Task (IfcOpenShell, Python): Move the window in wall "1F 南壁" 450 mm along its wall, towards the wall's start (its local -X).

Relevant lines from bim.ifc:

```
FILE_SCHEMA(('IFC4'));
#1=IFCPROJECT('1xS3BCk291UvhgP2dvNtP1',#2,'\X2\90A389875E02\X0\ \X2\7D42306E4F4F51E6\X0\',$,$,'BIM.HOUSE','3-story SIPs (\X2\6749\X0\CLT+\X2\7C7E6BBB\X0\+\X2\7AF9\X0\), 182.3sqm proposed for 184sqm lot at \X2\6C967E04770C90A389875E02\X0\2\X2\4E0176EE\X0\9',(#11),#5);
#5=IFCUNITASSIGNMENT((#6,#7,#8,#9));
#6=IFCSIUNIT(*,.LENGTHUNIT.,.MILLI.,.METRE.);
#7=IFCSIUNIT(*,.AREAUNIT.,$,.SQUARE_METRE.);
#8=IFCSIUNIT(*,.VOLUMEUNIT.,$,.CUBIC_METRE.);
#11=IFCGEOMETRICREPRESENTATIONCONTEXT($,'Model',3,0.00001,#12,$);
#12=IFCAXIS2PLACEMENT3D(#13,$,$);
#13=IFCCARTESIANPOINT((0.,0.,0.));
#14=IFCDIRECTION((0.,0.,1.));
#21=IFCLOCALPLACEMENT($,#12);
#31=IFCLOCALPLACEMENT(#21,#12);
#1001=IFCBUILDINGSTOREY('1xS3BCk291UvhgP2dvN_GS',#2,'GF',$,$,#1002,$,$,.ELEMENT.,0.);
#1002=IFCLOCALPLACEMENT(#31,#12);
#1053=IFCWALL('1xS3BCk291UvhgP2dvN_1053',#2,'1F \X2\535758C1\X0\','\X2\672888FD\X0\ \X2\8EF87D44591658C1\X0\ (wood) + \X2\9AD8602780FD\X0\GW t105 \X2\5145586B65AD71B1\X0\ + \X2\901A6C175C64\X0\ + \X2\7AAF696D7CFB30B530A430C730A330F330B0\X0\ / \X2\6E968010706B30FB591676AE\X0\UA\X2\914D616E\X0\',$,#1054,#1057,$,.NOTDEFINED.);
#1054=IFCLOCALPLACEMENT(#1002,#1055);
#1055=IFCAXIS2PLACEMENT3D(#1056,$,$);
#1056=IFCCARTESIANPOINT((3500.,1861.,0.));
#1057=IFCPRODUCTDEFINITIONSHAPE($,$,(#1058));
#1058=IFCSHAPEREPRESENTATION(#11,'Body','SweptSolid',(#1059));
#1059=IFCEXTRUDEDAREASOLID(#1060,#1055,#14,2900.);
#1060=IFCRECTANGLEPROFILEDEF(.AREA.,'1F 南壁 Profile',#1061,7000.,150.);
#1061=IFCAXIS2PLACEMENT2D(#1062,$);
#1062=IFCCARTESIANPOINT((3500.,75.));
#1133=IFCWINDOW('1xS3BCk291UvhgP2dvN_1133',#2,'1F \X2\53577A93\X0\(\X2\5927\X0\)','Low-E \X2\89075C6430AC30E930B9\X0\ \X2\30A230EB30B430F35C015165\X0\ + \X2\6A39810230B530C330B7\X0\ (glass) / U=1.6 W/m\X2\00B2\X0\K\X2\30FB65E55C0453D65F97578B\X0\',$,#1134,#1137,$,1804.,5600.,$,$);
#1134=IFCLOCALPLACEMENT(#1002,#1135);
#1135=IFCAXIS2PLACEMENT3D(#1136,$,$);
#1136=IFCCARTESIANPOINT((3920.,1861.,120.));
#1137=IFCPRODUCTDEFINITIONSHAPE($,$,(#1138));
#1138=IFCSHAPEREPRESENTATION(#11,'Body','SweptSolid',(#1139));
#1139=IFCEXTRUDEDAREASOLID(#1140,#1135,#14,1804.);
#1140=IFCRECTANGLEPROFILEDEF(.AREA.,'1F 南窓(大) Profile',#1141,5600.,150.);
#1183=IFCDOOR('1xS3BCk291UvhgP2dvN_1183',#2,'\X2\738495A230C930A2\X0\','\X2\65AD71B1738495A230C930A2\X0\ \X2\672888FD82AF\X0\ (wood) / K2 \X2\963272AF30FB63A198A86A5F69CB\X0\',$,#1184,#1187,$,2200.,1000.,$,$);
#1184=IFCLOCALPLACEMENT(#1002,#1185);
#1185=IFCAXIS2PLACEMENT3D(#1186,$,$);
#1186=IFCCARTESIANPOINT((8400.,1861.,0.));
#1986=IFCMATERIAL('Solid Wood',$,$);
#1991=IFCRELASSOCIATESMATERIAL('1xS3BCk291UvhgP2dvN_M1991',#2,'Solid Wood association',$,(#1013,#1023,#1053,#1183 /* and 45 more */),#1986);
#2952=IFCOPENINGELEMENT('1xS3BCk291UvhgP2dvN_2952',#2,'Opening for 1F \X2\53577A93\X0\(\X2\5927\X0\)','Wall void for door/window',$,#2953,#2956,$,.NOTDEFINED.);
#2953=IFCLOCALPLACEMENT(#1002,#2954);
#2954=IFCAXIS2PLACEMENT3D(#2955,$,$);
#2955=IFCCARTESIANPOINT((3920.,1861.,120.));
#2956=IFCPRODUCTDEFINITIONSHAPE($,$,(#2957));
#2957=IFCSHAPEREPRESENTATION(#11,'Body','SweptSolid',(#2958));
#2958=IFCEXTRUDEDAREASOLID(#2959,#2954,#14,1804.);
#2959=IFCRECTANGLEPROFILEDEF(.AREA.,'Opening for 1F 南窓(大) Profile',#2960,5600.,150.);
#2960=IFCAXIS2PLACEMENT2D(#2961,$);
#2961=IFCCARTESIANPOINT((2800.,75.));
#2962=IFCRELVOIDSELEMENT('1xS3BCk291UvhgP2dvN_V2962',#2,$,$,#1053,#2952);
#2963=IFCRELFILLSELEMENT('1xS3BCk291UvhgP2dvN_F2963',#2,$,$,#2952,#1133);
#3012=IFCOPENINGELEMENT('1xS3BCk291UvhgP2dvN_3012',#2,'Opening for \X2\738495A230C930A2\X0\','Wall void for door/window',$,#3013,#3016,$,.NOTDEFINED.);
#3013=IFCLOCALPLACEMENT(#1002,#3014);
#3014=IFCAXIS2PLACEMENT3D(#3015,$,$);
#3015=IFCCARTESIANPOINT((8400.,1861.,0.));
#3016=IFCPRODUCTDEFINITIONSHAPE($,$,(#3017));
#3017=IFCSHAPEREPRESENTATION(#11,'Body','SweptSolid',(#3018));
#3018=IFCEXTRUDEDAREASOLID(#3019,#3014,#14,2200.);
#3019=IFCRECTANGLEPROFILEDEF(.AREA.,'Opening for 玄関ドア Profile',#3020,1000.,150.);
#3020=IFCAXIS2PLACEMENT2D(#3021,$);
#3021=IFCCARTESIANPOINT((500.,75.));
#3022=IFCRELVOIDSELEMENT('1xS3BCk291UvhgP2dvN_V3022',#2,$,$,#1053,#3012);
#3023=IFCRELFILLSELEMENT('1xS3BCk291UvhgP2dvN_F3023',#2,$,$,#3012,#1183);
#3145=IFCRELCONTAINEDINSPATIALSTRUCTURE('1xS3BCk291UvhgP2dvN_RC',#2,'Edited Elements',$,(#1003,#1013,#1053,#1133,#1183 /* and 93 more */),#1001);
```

```python
import ifcopenshell
import ifcopenshell.api.geometry
import ifcopenshell.util.placement
import ifcopenshell.util.unit

model = ifcopenshell.open("bim.ifc")
unit_scale = ifcopenshell.util.unit.calculate_unit_scale(model)

window = model.by_guid("1xS3BCk291UvhgP2dvN_1133")
opening = window.FillsVoids[0].RelatingOpeningElement
wall = opening.VoidsElements[0].RelatingBuildingElement

wall_matrix = ifcopenshell.util.placement.get_local_placement(wall.ObjectPlacement)
shift = wall_matrix[:3, 0] * -0.45 / unit_scale
before = ifcopenshell.util.placement.get_local_placement(window.ObjectPlacement)[:3, 3].copy()

# The window is not placed relative to its opening, so move both.
for product in (opening, window):
    matrix = ifcopenshell.util.placement.get_local_placement(product.ObjectPlacement)
    matrix[:3, 3] += shift
    ifcopenshell.api.geometry.edit_object_placement(model, product=product, matrix=matrix, is_si=False)

after = ifcopenshell.util.placement.get_local_placement(window.ObjectPlacement)[:3, 3]
print("window moved by", (after - before).round(3) + 0.0)

model.write("bim_rev.ifc")
```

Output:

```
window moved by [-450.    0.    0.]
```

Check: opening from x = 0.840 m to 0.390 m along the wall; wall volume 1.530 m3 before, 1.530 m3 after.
